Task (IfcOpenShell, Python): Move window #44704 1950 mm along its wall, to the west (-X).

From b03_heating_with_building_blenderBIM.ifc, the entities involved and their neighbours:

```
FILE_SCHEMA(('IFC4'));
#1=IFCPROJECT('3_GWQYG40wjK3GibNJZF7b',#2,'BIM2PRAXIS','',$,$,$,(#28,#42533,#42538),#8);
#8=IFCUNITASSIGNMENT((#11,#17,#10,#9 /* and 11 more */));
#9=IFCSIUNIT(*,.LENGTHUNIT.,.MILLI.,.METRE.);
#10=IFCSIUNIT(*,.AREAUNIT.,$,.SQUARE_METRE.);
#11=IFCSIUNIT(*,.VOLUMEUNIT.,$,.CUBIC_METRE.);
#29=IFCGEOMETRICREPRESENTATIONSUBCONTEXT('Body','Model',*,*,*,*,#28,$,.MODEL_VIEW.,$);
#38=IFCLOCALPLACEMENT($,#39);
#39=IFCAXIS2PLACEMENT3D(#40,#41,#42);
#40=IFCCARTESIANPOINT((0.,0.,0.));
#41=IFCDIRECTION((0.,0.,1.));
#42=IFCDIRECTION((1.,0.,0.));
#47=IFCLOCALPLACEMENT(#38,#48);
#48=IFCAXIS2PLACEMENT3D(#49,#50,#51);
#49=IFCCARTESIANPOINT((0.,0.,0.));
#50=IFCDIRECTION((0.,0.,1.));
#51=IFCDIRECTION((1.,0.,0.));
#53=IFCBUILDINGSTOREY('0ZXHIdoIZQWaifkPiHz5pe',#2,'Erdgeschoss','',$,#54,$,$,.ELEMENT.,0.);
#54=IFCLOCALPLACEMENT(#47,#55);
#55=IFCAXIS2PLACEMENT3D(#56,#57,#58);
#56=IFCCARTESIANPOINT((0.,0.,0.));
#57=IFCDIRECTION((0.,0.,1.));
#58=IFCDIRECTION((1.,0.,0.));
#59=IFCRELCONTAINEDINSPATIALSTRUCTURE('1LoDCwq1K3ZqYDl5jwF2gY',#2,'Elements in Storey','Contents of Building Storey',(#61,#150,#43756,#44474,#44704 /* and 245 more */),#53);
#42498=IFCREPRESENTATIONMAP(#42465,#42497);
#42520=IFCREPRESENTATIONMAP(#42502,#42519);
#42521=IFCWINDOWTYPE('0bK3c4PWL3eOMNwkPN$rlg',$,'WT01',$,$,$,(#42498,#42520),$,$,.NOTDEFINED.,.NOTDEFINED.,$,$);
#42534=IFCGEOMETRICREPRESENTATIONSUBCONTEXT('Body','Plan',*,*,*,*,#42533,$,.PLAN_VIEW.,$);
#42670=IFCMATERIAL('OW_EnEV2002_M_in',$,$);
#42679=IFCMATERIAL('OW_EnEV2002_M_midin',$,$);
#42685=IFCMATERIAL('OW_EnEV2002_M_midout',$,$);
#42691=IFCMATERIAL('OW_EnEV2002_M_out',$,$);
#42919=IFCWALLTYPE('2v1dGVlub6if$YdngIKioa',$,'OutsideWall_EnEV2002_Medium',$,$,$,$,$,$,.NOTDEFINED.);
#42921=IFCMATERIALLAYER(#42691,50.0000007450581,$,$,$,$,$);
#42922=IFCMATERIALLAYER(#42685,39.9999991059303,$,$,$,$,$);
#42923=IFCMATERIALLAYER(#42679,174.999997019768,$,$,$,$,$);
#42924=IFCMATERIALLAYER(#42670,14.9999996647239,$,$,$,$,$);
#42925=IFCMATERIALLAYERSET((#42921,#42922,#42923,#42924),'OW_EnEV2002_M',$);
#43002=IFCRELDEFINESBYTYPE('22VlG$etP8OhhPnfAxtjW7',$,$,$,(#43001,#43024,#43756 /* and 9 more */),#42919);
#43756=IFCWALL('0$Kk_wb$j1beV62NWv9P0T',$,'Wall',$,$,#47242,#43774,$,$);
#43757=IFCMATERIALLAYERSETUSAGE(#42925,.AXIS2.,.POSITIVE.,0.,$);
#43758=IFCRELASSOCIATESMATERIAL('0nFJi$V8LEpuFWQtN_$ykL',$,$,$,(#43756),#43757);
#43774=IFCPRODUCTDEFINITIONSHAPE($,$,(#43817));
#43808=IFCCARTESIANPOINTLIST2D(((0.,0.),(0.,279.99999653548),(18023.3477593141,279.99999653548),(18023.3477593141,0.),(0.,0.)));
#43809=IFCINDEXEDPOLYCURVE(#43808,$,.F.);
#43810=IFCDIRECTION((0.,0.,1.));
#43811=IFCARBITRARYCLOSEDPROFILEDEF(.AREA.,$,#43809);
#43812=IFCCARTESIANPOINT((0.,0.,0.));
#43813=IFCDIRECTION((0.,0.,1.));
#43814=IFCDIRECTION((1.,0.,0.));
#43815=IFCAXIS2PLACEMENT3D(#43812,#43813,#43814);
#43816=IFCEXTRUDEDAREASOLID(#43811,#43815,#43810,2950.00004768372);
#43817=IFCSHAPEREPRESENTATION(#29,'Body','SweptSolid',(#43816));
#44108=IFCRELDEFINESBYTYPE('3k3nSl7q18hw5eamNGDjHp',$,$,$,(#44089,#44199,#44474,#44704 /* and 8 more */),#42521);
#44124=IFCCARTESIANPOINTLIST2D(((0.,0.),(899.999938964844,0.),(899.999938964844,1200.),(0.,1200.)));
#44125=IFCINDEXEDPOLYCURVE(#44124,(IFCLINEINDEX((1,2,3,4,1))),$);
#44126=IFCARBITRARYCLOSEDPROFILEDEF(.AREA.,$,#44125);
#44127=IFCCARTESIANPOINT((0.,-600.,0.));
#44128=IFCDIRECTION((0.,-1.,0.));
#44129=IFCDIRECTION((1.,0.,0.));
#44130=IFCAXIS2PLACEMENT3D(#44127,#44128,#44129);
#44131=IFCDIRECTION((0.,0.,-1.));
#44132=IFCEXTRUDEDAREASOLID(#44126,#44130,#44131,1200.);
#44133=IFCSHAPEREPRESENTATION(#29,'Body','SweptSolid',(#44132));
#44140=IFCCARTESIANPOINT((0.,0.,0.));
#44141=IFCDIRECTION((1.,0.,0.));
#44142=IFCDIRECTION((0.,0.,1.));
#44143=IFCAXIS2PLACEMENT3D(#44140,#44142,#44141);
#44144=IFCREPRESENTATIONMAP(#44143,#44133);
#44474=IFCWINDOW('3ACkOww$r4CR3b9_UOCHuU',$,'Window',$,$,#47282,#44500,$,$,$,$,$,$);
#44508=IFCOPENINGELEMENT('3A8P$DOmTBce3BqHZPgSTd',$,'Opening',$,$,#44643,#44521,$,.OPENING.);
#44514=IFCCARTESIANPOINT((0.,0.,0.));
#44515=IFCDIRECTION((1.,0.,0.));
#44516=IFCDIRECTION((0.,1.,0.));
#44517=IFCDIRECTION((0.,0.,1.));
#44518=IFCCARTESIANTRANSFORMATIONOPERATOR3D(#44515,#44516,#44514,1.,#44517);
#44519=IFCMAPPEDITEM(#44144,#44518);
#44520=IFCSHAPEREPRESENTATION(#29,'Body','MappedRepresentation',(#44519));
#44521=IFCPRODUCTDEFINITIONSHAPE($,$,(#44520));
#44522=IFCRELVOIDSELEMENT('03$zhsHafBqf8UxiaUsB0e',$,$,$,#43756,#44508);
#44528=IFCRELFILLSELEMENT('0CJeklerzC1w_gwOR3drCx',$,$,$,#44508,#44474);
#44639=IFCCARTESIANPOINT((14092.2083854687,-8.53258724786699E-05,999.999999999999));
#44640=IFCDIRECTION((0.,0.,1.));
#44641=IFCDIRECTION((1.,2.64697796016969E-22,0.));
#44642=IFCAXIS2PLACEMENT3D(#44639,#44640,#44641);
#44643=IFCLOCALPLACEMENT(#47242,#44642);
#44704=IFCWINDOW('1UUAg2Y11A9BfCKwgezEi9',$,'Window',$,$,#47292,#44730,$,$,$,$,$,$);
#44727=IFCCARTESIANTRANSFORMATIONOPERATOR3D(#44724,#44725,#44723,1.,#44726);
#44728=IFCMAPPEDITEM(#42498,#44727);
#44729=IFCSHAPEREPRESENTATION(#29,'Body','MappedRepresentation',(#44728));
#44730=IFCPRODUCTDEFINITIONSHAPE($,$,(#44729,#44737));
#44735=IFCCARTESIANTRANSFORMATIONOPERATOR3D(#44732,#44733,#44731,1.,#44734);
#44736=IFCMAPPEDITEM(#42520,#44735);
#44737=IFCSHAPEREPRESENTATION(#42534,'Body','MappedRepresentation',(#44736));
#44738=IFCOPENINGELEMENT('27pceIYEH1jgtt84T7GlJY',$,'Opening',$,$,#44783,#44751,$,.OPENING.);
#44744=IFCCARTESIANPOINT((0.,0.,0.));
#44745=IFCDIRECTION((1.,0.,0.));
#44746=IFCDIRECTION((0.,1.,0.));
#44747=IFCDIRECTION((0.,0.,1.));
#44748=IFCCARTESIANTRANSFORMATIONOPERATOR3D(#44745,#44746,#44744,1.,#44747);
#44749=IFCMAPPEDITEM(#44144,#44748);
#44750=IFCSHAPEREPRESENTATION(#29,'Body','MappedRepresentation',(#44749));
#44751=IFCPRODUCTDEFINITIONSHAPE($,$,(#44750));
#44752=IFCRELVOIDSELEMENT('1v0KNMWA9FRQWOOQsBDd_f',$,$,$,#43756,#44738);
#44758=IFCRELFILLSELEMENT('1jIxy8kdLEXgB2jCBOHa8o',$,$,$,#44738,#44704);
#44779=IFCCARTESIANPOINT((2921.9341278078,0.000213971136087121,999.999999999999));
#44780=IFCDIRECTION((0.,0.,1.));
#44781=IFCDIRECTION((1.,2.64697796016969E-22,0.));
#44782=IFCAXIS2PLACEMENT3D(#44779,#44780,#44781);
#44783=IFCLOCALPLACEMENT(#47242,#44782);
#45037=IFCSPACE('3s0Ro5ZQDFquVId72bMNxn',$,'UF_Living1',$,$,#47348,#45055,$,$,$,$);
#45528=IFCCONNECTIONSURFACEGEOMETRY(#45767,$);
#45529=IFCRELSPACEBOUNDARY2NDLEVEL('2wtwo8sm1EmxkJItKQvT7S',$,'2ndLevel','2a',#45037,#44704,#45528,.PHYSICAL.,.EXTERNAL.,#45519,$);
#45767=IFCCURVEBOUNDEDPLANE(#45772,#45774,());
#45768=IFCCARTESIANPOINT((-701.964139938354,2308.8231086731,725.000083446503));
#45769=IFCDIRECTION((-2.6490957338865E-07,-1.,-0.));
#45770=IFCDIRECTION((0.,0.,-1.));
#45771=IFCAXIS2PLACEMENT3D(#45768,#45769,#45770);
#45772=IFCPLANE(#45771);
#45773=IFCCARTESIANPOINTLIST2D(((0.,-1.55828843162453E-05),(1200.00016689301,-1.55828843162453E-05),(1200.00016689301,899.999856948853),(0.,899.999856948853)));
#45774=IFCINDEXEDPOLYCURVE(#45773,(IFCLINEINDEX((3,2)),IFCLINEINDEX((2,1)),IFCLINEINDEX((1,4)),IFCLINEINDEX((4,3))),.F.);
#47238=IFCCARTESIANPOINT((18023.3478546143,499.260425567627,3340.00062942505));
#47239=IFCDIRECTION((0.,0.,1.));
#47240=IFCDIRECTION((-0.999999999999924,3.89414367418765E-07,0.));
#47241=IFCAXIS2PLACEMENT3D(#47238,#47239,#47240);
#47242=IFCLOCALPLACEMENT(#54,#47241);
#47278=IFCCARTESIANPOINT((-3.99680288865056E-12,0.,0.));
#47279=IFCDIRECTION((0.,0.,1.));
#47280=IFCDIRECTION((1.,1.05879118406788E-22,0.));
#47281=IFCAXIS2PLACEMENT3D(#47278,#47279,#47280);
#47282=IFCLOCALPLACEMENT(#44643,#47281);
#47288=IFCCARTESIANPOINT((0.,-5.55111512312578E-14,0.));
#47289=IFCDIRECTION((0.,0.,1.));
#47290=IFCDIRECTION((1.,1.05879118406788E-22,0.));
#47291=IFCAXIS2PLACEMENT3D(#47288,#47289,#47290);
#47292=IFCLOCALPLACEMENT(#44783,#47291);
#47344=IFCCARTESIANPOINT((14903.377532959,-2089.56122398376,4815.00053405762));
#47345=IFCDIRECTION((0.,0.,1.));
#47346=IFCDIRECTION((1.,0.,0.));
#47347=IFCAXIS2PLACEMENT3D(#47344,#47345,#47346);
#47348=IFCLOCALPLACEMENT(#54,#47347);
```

```python
import numpy as np
import ifcopenshell
import ifcopenshell.api.geometry
import ifcopenshell.util.placement
import ifcopenshell.util.unit

model = ifcopenshell.open("b03_heating_with_building_blenderBIM.ifc")
unit_scale = ifcopenshell.util.unit.calculate_unit_scale(model)

window = model.by_guid("1UUAg2Y11A9BfCKwgezEi9")
opening = window.FillsVoids[0].RelatingOpeningElement
wall = opening.VoidsElements[0].RelatingBuildingElement

wall_matrix = ifcopenshell.util.placement.get_local_placement(wall.ObjectPlacement)
shift = wall_matrix[:3, 0] * 1.95 / unit_scale
before = ifcopenshell.util.placement.get_local_placement(window.ObjectPlacement)[:3, 3].copy()

# The window is placed relative to its opening, so it follows when the opening moves.
matrix = ifcopenshell.util.placement.get_local_placement(opening.ObjectPlacement)
matrix[:3, 3] += shift
ifcopenshell.api.geometry.edit_object_placement(
    model, product=opening, matrix=matrix, is_si=False, should_transform_children=True
)

# Space boundary surfaces are stored in each space's coordinates; move them too.
for rel in window.ProvidesBoundaries:
    if not rel.ConnectionGeometry:
        continue
    surface = rel.ConnectionGeometry.SurfaceOnRelatingElement.BasisSurface
    space_matrix = ifcopenshell.util.placement.get_local_placement(rel.RelatingSpace.ObjectPlacement)
    point = np.array(surface.Position.Location.Coordinates) + space_matrix[:3, :3].T @ shift
    surface.Position = model.createIfcAxis2Placement3D(
        model.createIfcCartesianPoint(point.tolist()), surface.Position.Axis, surface.Position.RefDirection
    )

after = ifcopenshell.util.placement.get_local_placement(window.ObjectPlacement)[:3, 3]
print("window moved by", (after - before).round(3) + 0.0)

model.write("b03_heating_with_building_blenderBIM-out.ifc")
```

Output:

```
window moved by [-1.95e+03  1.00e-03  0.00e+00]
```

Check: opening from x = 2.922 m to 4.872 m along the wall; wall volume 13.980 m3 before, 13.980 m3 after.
